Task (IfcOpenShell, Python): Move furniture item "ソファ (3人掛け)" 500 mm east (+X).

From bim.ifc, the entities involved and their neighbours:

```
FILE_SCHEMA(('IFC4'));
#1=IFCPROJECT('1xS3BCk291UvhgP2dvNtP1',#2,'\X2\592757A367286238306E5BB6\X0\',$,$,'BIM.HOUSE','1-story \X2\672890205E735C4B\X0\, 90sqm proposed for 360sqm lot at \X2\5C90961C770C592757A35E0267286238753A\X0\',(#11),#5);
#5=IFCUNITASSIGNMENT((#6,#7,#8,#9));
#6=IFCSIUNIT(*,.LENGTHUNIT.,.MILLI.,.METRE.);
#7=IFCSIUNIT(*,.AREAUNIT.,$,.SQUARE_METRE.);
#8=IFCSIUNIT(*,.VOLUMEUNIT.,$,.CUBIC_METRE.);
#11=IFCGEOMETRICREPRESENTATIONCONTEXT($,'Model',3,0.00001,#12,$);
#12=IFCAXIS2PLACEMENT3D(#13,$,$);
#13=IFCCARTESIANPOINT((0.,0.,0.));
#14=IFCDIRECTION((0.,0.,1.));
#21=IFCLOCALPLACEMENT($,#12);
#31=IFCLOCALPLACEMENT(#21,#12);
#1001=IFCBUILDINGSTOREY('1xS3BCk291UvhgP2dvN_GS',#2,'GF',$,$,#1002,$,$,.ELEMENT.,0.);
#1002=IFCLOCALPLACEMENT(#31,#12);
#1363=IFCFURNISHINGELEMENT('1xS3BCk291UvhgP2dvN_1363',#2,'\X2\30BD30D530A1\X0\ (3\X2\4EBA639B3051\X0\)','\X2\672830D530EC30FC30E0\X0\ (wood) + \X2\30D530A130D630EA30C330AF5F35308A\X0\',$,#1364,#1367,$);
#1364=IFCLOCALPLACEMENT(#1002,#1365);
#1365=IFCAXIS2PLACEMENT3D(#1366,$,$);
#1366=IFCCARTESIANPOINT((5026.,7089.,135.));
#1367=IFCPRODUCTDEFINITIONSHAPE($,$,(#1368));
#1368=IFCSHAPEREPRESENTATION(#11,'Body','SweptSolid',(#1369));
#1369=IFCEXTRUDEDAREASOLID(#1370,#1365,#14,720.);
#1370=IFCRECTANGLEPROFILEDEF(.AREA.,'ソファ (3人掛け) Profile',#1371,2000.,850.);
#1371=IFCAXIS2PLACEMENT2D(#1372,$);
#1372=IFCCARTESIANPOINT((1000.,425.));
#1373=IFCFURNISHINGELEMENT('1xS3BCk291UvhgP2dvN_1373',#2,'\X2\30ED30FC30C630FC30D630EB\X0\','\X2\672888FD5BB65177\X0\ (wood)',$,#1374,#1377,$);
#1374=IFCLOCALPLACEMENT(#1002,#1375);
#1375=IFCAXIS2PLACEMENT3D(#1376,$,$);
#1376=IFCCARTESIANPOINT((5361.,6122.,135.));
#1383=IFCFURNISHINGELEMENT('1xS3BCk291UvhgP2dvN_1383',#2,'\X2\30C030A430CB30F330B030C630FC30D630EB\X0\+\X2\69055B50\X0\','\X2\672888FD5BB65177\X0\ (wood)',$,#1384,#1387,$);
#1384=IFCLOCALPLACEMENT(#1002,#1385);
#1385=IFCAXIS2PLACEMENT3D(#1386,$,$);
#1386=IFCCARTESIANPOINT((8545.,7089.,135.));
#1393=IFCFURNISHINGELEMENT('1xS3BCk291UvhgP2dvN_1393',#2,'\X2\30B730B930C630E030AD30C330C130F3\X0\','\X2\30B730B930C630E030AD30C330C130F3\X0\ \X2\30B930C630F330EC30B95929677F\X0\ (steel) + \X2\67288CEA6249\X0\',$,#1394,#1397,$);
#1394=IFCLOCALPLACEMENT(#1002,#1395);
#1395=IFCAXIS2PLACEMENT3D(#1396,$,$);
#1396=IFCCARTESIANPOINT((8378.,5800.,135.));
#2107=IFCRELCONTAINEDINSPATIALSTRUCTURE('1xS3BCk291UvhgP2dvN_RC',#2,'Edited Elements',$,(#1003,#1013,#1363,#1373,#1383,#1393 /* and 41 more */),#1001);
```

```python
import ifcopenshell
import ifcopenshell.api.geometry
import ifcopenshell.util.placement
import ifcopenshell.util.unit

model = ifcopenshell.open("bim.ifc")
unit_scale = ifcopenshell.util.unit.calculate_unit_scale(model)

item = model.by_guid("1xS3BCk291UvhgP2dvN_1363")
matrix = ifcopenshell.util.placement.get_local_placement(item.ObjectPlacement)
matrix[0, 3] += 0.5 / unit_scale
ifcopenshell.api.geometry.edit_object_placement(model, product=item, matrix=matrix, is_si=False)

print(ifcopenshell.util.placement.get_local_placement(item.ObjectPlacement).round(3) + 0.0)

model.write("bim_edited.ifc")
```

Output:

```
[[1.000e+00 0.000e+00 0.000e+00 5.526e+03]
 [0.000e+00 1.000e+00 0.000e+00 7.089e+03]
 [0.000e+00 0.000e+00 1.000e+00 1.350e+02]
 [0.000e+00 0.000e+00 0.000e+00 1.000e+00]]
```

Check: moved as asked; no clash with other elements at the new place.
